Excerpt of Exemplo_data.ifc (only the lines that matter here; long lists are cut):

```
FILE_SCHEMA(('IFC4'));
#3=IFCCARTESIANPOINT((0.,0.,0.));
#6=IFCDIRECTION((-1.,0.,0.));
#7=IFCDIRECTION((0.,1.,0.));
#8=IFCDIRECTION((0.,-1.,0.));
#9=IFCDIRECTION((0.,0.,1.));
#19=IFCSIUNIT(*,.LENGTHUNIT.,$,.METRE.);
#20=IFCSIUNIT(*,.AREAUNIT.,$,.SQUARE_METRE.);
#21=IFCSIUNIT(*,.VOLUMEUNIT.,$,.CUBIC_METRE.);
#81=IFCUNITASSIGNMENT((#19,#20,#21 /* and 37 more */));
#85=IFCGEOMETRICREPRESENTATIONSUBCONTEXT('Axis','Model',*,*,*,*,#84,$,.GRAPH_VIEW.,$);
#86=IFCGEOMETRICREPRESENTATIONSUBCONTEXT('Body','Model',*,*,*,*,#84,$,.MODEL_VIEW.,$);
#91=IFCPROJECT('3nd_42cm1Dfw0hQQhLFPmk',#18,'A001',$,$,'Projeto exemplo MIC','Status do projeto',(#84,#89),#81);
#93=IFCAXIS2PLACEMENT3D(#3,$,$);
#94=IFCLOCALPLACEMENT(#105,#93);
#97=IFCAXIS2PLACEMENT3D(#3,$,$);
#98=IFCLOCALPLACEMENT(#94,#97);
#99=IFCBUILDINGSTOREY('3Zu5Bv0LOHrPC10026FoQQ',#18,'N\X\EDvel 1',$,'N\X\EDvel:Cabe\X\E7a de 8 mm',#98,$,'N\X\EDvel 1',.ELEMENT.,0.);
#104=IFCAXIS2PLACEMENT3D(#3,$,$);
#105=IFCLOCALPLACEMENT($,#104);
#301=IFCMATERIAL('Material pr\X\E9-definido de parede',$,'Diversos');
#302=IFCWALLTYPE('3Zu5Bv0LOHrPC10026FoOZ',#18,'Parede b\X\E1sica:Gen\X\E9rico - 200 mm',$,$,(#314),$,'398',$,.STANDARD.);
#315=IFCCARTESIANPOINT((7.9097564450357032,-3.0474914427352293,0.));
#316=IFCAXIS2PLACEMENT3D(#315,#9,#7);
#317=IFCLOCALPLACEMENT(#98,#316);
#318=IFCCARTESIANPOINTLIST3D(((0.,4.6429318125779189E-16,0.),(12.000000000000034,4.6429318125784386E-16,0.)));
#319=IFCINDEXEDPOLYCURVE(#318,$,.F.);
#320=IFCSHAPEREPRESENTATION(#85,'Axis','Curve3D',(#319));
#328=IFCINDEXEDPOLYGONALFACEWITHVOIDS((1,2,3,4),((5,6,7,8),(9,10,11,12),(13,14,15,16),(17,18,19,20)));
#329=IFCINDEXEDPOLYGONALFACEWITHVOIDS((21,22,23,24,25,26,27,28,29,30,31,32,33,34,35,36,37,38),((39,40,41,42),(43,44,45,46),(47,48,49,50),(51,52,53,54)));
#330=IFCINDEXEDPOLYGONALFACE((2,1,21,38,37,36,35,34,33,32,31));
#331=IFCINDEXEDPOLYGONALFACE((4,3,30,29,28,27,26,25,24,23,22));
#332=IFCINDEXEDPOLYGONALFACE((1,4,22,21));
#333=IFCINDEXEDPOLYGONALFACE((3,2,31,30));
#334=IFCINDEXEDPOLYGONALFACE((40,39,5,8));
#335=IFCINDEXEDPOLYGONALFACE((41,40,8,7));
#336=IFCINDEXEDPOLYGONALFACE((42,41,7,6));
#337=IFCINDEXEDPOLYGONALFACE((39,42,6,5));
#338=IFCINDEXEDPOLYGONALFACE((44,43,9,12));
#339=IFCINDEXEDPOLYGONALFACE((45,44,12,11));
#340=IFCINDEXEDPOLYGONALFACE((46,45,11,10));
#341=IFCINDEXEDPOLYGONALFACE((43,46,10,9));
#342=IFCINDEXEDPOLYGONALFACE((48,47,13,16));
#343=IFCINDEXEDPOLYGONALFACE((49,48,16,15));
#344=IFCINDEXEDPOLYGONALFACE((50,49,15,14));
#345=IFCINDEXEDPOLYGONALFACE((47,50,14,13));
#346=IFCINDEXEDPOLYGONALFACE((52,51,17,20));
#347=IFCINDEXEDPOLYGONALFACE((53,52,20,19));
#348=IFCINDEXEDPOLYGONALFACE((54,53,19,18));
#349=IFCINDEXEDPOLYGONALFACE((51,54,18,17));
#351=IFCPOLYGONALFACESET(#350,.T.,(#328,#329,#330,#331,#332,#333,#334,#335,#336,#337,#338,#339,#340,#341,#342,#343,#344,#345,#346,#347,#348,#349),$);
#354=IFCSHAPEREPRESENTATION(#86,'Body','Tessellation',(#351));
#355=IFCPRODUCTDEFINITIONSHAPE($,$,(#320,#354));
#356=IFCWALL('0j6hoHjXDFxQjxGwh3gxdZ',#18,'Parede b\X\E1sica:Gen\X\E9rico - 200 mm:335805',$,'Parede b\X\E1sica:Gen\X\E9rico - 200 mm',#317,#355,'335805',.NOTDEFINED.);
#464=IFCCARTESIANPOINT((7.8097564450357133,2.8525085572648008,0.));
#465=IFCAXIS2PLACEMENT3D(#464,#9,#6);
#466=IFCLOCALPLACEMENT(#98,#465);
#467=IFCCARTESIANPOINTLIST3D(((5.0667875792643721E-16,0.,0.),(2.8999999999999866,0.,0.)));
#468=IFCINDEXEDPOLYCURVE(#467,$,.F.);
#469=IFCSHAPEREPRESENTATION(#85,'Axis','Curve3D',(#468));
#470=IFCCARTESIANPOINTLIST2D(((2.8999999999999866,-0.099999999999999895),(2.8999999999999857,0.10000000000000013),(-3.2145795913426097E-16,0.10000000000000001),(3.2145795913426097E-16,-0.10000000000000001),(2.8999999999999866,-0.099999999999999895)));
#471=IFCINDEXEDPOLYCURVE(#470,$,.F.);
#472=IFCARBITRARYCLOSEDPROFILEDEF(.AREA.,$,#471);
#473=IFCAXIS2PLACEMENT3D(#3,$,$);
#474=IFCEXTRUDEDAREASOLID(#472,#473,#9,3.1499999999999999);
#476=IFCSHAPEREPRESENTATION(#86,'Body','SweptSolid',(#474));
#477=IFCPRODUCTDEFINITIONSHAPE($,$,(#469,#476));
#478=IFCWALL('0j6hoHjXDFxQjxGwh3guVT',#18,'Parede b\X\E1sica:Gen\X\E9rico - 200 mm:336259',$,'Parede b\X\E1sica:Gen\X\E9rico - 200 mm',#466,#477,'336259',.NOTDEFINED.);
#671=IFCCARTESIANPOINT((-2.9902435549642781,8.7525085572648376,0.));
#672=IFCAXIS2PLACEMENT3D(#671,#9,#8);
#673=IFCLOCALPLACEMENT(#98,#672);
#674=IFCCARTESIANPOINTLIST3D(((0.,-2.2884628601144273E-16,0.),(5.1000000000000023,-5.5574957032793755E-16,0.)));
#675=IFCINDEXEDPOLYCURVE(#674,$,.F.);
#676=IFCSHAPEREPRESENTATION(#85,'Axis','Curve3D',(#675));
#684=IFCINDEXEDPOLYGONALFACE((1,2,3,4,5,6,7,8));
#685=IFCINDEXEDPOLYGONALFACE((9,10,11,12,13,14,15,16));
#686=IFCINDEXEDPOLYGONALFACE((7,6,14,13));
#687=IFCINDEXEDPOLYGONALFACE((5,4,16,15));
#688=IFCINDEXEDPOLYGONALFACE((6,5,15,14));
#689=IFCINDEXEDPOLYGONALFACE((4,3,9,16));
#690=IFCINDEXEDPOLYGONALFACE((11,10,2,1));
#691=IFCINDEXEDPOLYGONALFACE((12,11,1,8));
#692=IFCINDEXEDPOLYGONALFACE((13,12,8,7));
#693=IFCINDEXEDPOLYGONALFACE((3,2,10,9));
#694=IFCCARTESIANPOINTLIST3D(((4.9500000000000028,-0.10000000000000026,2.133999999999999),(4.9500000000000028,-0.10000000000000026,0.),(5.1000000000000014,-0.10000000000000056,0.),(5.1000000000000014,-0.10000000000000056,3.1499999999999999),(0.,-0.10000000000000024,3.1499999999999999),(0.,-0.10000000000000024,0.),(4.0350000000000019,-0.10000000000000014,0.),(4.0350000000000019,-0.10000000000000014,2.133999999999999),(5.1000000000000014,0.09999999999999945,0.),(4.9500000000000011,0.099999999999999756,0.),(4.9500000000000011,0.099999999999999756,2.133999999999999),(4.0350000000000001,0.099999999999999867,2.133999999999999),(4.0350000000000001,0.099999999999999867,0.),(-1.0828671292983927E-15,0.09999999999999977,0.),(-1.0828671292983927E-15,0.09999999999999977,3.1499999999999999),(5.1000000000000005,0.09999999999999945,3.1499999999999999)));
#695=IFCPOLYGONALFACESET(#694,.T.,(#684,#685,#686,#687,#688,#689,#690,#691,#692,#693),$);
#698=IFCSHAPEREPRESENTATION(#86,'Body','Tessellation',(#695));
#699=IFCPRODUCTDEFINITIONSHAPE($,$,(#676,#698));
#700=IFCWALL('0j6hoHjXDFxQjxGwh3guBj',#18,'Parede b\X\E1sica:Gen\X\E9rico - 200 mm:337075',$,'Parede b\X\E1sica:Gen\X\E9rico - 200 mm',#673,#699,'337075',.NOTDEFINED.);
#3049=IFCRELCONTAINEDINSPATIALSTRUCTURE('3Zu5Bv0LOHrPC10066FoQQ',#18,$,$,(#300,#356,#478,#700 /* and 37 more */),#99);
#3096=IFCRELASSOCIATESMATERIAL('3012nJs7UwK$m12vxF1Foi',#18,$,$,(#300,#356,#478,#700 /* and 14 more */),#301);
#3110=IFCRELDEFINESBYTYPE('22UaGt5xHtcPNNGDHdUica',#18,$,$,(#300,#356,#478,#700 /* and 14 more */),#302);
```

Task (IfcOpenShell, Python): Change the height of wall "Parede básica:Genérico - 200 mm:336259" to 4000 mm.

```python
import ifcopenshell
import ifcopenshell.geom
import ifcopenshell.util.representation
import ifcopenshell.util.shape

model = ifcopenshell.open("Exemplo_data.ifc")
settings = ifcopenshell.geom.settings()


def volume(element):
    """Net volume in cubic metres, openings subtracted."""
    shape = ifcopenshell.geom.create_shape(settings, element)
    return ifcopenshell.util.shape.get_volume(shape.geometry)


wall = model.by_guid("0j6hoHjXDFxQjxGwh3guVT")
before = volume(wall)

body = ifcopenshell.util.representation.get_representation(wall, "Model", "Body")
solid = body.Items[0]
old_height = solid.Depth
solid.Depth = 4.0
after = volume(wall)

print(f"height {old_height:g} -> {solid.Depth:g}, volume {before:.3f} -> {after:.3f} m3")

model.write("Exemplo_data_rev.ifc")
```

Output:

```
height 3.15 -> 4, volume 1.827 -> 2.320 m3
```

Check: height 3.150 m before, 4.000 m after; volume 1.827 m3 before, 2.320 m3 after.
